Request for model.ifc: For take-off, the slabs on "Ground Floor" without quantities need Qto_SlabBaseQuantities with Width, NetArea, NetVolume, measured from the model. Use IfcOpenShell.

First a look at what the model holds.

```python
import ifcopenshell
import ifcopenshell.util.element
import ifcopenshell.util.unit

model = ifcopenshell.open("model.ifc")
print(model.schema)
for unit_type in ("LENGTHUNIT", "AREAUNIT", "VOLUMEUNIT"):
    print(unit_type, ifcopenshell.util.unit.calculate_unit_scale(model, unit_type))
storey = next(s for s in model.by_type("IfcBuildingStorey") if s.Name == "Ground Floor")
slabs = [e for e in ifcopenshell.util.element.get_decomposition(storey) if e.is_a("IfcSlab")]
for e in sorted(slabs, key=lambda e: e.id()):
    print(e.id(), e.is_a(), e.Name, list(ifcopenshell.util.element.get_psets(e, qtos_only=True)), sep=" | ")
```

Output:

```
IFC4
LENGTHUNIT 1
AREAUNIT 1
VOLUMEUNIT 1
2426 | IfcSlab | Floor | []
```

```python
import ifcopenshell
import ifcopenshell.api.pset
import ifcopenshell.geom
import ifcopenshell.util.element
import ifcopenshell.util.shape
import ifcopenshell.util.unit

model = ifcopenshell.open("model.ifc")
unit_scale = ifcopenshell.util.unit.calculate_unit_scale(model)
area_scale = ifcopenshell.util.unit.calculate_unit_scale(model, "AREAUNIT")
volume_scale = ifcopenshell.util.unit.calculate_unit_scale(model, "VOLUMEUNIT")
settings = ifcopenshell.geom.settings()

storey = next(s for s in model.by_type("IfcBuildingStorey") if s.Name == "Ground Floor")
slabs = [e for e in ifcopenshell.util.element.get_decomposition(storey) if e.is_a("IfcSlab")]

for e in sorted(slabs, key=lambda e: e.id()):
    if ifcopenshell.util.element.get_psets(e, qtos_only=True, should_inherit=False):
        continue
    # Geometry comes back in metres, in the element's own axes.
    shape = ifcopenshell.geom.create_shape(settings, e)
    values = {
        "Width": ifcopenshell.util.shape.get_z(shape.geometry) / unit_scale,
        "NetArea": ifcopenshell.util.shape.get_footprint_area(shape.geometry) / area_scale,
        "NetVolume": ifcopenshell.util.shape.get_volume(shape.geometry) / volume_scale,
    }
    qto = ifcopenshell.api.pset.add_qto(model, product=e, name="Qto_SlabBaseQuantities")
    ifcopenshell.api.pset.edit_qto(model, qto=qto, properties=values)
    print(e.id(), {k: round(v, 3) for k, v in values.items()})

model.write("model-out.ifc")
```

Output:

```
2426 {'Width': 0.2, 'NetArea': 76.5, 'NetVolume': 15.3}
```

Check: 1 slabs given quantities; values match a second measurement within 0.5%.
